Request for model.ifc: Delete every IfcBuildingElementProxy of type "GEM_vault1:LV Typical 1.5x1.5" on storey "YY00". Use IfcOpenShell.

First a look at what the model holds.

```python
import ifcopenshell
import ifcopenshell.util.element

model = ifcopenshell.open("model.ifc")
print(model.schema)
storey = next(s for s in model.by_type("IfcBuildingStorey") if s.Name == "YY00")
proxies = [e for e in ifcopenshell.util.element.get_decomposition(storey) if e.is_a("IfcBuildingElementProxy")]
seen = {}
for e in proxies:
    element_type = ifcopenshell.util.element.get_type(e)
    name = element_type.Name if element_type not in (None, e) else None
    seen[name] = seen.get(name, 0) + 1
for name, count in sorted(seen.items(), key=str):
    print(count, "x", name)
```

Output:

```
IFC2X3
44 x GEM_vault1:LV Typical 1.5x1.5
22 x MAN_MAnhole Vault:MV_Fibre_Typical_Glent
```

```python
import ifcopenshell
import ifcopenshell.api.root
import ifcopenshell.util.element

model = ifcopenshell.open("model.ifc")

storey = next(s for s in model.by_type("IfcBuildingStorey") if s.Name == "YY00")
proxies = [e for e in ifcopenshell.util.element.get_decomposition(storey) if e.is_a("IfcBuildingElementProxy")]
targets = [e for e in proxies if (t := ifcopenshell.util.element.get_type(e)) not in (None, e) and t.Name == "GEM_vault1:LV Typical 1.5x1.5"]

for e in targets:
    ifcopenshell.api.root.remove_product(model, product=e)
print(len(targets), "removed")

model.write("model_v2.ifc")
```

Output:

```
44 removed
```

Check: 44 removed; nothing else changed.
